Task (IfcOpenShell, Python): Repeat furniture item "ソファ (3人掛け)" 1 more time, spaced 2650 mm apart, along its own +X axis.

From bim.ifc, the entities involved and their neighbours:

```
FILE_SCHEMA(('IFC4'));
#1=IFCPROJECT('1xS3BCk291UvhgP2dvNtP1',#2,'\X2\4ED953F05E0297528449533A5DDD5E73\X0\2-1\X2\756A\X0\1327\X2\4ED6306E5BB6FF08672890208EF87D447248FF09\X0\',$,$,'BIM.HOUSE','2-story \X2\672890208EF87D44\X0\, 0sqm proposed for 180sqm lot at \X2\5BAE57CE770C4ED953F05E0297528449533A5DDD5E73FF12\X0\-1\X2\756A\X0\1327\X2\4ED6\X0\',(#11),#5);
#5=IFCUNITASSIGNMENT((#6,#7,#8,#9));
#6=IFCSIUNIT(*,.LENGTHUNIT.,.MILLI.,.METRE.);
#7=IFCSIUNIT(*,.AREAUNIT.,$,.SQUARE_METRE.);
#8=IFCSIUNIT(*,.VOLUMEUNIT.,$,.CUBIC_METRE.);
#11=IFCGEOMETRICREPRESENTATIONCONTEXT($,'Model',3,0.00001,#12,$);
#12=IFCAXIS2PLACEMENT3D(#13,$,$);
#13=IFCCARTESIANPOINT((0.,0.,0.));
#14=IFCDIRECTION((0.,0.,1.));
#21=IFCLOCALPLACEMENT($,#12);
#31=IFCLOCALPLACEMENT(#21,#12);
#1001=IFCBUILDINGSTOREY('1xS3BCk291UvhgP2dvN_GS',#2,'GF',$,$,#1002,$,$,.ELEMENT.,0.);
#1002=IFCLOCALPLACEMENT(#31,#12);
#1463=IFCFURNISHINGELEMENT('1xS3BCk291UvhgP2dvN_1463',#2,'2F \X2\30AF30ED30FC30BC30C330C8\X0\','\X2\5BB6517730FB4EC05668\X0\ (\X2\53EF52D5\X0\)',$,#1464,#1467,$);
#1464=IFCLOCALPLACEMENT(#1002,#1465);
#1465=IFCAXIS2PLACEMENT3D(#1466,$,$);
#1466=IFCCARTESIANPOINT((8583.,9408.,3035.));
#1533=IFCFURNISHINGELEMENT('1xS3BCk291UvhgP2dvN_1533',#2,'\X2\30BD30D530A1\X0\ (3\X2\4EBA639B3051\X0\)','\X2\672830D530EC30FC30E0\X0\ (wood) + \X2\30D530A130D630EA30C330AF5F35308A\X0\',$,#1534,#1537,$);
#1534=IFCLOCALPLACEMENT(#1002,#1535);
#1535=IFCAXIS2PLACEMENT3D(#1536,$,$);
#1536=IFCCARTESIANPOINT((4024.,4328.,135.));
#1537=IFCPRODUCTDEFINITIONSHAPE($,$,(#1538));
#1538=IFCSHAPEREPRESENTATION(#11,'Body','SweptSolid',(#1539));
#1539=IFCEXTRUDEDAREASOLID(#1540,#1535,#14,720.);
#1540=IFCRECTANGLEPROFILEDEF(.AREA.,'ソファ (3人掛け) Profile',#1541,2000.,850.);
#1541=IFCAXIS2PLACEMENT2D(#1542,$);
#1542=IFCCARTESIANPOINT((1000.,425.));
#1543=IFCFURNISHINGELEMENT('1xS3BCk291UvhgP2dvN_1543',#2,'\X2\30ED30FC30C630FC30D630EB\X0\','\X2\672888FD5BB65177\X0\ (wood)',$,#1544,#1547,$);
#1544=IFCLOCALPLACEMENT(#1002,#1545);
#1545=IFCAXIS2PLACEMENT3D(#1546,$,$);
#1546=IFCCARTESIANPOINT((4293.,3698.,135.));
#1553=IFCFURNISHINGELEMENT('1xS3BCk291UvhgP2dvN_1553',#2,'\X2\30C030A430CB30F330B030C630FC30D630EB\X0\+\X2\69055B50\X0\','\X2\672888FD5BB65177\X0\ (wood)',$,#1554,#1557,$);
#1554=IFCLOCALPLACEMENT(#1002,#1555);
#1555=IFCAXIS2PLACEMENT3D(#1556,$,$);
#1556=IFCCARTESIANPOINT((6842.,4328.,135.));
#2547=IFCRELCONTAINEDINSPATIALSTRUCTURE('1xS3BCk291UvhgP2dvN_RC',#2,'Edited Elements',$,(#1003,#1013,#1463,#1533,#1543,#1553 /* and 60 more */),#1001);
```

```python
import ifcopenshell
import ifcopenshell.api.geometry
import ifcopenshell.api.root
import ifcopenshell.util.element
import ifcopenshell.util.placement

model = ifcopenshell.open("bim.ifc")


def reuse_history(source, copy):
    """copy_class also copies each property set's owner history, people and application; keep the originals."""
    for rel in copy.IsDefinedBy:
        if rel.is_a("IfcRelDefinesByProperties") and (history := rel.RelatingPropertyDefinition.OwnerHistory):
            rel.RelatingPropertyDefinition.OwnerHistory = source.OwnerHistory
            ifcopenshell.util.element.remove_deep2(model, history)


source = model.by_guid("1xS3BCk291UvhgP2dvN_1533")
base = ifcopenshell.util.placement.get_local_placement(source.ObjectPlacement)
step = base[:3, 0] * 2650.0

for i in range(1, 2):
    copy = ifcopenshell.api.root.copy_class(model, product=source)
    copy.Representation = ifcopenshell.util.element.copy_deep(
        model, source.Representation, exclude=["IfcGeometricRepresentationContext", "IfcRepresentationMap"]
    )
    reuse_history(source, copy)
    matrix = base.copy()
    matrix[:3, 3] += i * step
    print("added at", matrix[:3, 3].round(3) + 0.0)
    ifcopenshell.api.geometry.edit_object_placement(model, product=copy, matrix=matrix, is_si=False)

model.write("bim-out.ifc")
```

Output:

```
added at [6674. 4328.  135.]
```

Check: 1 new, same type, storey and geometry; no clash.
